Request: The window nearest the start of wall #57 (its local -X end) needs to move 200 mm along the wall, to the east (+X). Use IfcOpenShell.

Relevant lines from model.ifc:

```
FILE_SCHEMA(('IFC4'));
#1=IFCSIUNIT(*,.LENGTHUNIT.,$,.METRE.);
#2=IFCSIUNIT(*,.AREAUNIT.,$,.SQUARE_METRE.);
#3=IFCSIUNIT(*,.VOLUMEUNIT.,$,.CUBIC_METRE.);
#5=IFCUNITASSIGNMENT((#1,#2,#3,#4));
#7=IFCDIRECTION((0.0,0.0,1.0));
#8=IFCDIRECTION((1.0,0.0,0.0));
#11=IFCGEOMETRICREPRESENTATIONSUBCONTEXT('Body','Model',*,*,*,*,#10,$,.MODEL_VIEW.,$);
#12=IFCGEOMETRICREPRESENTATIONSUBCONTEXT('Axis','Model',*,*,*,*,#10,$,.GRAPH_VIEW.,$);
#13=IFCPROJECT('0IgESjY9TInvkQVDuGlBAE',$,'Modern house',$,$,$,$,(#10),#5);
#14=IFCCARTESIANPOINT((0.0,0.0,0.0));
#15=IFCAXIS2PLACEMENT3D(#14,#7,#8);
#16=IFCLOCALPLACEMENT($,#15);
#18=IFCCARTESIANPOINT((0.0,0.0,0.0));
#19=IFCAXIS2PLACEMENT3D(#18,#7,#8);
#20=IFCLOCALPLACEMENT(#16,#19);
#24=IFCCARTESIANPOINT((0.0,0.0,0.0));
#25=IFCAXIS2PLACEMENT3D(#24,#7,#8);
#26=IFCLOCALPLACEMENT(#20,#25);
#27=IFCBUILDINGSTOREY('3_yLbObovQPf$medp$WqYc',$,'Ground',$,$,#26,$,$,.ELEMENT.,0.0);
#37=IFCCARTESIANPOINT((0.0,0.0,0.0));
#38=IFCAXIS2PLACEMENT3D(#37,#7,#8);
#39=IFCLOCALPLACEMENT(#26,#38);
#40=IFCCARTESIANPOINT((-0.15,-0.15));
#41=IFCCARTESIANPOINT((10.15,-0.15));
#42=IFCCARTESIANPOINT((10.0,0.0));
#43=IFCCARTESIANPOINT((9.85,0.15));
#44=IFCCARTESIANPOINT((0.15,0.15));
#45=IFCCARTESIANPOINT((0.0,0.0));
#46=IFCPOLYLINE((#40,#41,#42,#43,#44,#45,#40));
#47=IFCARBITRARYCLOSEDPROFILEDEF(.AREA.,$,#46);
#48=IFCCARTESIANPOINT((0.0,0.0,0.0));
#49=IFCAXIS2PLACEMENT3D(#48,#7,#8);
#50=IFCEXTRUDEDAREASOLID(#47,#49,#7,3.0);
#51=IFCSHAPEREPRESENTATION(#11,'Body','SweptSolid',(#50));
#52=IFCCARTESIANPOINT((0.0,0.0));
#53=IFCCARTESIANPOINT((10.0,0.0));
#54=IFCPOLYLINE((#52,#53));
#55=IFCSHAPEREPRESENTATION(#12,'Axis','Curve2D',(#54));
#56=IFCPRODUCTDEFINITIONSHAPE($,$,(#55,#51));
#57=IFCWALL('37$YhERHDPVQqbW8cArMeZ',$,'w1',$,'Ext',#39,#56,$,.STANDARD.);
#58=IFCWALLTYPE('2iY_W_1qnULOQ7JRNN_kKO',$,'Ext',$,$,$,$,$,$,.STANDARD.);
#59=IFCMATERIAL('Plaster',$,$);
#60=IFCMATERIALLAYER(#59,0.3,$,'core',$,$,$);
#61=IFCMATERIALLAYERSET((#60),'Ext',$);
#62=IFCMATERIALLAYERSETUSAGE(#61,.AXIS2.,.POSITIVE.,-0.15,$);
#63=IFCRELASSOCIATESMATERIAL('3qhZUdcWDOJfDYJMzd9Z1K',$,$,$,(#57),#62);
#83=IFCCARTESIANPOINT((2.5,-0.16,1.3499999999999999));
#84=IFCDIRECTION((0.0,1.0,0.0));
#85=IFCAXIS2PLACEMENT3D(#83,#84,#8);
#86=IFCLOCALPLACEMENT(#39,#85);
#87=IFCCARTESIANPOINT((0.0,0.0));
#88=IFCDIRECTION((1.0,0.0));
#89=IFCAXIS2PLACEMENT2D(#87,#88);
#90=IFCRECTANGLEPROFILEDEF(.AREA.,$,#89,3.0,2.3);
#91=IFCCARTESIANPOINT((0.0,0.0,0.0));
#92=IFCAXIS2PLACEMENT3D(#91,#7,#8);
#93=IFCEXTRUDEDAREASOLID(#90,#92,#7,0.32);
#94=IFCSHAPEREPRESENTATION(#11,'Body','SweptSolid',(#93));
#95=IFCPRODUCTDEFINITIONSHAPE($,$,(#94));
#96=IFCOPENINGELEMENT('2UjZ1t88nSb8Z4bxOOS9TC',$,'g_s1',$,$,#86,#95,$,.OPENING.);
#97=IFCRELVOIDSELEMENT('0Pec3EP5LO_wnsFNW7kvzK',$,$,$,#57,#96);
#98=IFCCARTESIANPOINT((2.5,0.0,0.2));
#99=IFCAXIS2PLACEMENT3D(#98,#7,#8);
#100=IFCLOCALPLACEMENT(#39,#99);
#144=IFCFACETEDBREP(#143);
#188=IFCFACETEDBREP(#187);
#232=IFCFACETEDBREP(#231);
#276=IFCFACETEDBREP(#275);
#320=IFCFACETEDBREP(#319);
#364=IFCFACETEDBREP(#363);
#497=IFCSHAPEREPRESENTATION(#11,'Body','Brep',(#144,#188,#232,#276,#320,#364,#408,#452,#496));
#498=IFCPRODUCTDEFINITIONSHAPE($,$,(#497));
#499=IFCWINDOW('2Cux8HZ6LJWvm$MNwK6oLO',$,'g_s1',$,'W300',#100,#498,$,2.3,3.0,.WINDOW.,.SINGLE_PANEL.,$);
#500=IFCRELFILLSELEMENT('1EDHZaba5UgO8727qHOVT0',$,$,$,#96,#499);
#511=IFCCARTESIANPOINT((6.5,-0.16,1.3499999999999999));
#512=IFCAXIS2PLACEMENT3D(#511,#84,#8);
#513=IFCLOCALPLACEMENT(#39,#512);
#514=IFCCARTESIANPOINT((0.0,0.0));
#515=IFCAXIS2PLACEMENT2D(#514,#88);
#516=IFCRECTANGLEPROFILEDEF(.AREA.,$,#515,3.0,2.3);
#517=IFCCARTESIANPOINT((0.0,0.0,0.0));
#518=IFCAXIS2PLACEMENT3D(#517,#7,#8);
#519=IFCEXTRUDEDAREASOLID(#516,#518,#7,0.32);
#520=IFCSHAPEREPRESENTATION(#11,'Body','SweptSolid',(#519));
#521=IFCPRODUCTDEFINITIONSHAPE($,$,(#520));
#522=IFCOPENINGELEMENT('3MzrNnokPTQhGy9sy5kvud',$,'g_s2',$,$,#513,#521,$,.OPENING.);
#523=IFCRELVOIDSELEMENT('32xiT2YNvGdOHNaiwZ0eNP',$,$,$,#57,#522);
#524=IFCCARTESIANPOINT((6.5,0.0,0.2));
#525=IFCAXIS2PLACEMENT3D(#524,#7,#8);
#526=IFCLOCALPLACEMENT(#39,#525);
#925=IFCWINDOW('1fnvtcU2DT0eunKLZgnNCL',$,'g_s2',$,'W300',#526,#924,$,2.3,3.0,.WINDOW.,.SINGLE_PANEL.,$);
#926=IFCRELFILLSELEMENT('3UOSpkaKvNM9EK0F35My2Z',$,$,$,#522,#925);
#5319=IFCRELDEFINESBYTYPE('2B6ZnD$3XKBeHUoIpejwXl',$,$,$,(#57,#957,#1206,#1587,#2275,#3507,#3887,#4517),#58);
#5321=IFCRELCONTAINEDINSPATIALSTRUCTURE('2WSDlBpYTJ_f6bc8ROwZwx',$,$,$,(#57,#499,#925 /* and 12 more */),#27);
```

```python
import ifcopenshell
import ifcopenshell.api.geometry
import ifcopenshell.util.placement
import ifcopenshell.util.unit

model = ifcopenshell.open("model.ifc")
unit_scale = ifcopenshell.util.unit.calculate_unit_scale(model)

window = model.by_id(499)
opening = window.FillsVoids[0].RelatingOpeningElement
wall = opening.VoidsElements[0].RelatingBuildingElement

wall_matrix = ifcopenshell.util.placement.get_local_placement(wall.ObjectPlacement)
shift = wall_matrix[:3, 0] * 0.2 / unit_scale
before = ifcopenshell.util.placement.get_local_placement(window.ObjectPlacement)[:3, 3].copy()

# The window is not placed relative to its opening, so move both.
for product in (opening, window):
    matrix = ifcopenshell.util.placement.get_local_placement(product.ObjectPlacement)
    matrix[:3, 3] += shift
    ifcopenshell.api.geometry.edit_object_placement(model, product=product, matrix=matrix, is_si=False)

after = ifcopenshell.util.placement.get_local_placement(window.ObjectPlacement)[:3, 3]
print("window moved by", (after - before).round(3) + 0.0)

model.write("model_v2.ifc")
```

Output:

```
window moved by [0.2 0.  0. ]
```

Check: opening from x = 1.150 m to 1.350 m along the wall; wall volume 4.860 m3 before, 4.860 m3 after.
